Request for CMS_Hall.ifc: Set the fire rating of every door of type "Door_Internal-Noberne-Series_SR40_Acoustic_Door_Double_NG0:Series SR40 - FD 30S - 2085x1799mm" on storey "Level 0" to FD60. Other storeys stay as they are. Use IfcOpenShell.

First a look at what the model holds.

```python
import ifcopenshell
import ifcopenshell.util.element

model = ifcopenshell.open("CMS_Hall.ifc")
print(model.schema)
storey = next(s for s in model.by_type("IfcBuildingStorey") if s.Name == "Level 0")
doors = [e for e in ifcopenshell.util.element.get_decomposition(storey) if e.is_a("IfcDoor")]
seen = {}
for e in doors:
    element_type = ifcopenshell.util.element.get_type(e)
    key = (element_type.Name if element_type != e and element_type else None, ifcopenshell.util.element.get_pset(e, "Pset_DoorCommon", "FireRating"))
    seen[key] = seen.get(key, 0) + 1
for (name, value), count in sorted(seen.items(), key=str):
    print(count, "x", name, "|", value)
```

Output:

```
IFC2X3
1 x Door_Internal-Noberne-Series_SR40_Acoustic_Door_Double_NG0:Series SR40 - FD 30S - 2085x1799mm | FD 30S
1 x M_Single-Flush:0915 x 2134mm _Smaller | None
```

```python
import ifcopenshell
import ifcopenshell.api.pset
import ifcopenshell.util.element

model = ifcopenshell.open("CMS_Hall.ifc")

storey = next(s for s in model.by_type("IfcBuildingStorey") if s.Name == "Level 0")
doors = [e for e in ifcopenshell.util.element.get_decomposition(storey) if e.is_a("IfcDoor")]

count = 0
for e in doors:
    element_type = ifcopenshell.util.element.get_type(e)
    if element_type in (None, e) or element_type.Name != "Door_Internal-Noberne-Series_SR40_Acoustic_Door_Double_NG0:Series SR40 - FD 30S - 2085x1799mm":
        continue
    # add_pset returns the element's existing set when there is one.
    pset = ifcopenshell.api.pset.add_pset(model, product=e, name="Pset_DoorCommon")
    ifcopenshell.api.pset.edit_pset(model, pset=pset, properties={"FireRating": "FD60"})
    count += 1

print(count, "doors updated")

model.write("CMS_Hall_updated.ifc")
```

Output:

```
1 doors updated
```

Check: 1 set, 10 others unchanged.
